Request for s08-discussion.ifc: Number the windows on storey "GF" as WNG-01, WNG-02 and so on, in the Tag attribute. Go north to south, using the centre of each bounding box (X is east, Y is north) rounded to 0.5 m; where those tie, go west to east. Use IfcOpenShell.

First a look at what the model holds.

```python
import ifcopenshell
import ifcopenshell.util.element
import ifcopenshell.util.placement

model = ifcopenshell.open("s08-discussion.ifc")
print(model.schema)
storey = next(s for s in model.by_type("IfcBuildingStorey") if s.Name == "GF")
windows = [e for e in ifcopenshell.util.element.get_decomposition(storey) if e.is_a("IfcWindow")]
for e in sorted(windows, key=lambda e: e.id()):
    origin = ifcopenshell.util.placement.get_local_placement(e.ObjectPlacement)[:3, 3]
    print(e.id(), e.Tag, e.Name, origin.round(2) + 0.0, sep=" | ")
```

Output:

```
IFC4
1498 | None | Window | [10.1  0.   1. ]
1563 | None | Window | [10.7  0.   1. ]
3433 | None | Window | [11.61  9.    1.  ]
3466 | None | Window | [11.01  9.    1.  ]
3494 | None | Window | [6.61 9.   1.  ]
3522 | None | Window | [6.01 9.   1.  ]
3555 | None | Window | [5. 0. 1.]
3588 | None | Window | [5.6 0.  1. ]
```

```python
import ifcopenshell
import ifcopenshell.geom
import ifcopenshell.util.element
import ifcopenshell.util.shape

model = ifcopenshell.open("s08-discussion.ifc")
settings = ifcopenshell.geom.settings()
settings.set("use-world-coords", True)


def centre(element):
    shape = ifcopenshell.geom.create_shape(settings, element)
    return ifcopenshell.util.shape.get_bbox_centroid(shape.geometry)


storey = next(s for s in model.by_type("IfcBuildingStorey") if s.Name == "GF")
windows = [e for e in ifcopenshell.util.element.get_decomposition(storey) if e.is_a("IfcWindow")]

# Insertion points can sit at a corner or the storey origin, so sort by the geometry (in metres).
centres = {e: centre(e) for e in windows}
windows.sort(key=lambda e: (-round(centres[e][1] / 0.5), centres[e][0]))

for i, e in enumerate(windows, start=1):
    number = f"WNG-{i:02d}"
    e.Tag = number
    print(e.id(), number)

model.write("s08-discussion_rev.ifc")
```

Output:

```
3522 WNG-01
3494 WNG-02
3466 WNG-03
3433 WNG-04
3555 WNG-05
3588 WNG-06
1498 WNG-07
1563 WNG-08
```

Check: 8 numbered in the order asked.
